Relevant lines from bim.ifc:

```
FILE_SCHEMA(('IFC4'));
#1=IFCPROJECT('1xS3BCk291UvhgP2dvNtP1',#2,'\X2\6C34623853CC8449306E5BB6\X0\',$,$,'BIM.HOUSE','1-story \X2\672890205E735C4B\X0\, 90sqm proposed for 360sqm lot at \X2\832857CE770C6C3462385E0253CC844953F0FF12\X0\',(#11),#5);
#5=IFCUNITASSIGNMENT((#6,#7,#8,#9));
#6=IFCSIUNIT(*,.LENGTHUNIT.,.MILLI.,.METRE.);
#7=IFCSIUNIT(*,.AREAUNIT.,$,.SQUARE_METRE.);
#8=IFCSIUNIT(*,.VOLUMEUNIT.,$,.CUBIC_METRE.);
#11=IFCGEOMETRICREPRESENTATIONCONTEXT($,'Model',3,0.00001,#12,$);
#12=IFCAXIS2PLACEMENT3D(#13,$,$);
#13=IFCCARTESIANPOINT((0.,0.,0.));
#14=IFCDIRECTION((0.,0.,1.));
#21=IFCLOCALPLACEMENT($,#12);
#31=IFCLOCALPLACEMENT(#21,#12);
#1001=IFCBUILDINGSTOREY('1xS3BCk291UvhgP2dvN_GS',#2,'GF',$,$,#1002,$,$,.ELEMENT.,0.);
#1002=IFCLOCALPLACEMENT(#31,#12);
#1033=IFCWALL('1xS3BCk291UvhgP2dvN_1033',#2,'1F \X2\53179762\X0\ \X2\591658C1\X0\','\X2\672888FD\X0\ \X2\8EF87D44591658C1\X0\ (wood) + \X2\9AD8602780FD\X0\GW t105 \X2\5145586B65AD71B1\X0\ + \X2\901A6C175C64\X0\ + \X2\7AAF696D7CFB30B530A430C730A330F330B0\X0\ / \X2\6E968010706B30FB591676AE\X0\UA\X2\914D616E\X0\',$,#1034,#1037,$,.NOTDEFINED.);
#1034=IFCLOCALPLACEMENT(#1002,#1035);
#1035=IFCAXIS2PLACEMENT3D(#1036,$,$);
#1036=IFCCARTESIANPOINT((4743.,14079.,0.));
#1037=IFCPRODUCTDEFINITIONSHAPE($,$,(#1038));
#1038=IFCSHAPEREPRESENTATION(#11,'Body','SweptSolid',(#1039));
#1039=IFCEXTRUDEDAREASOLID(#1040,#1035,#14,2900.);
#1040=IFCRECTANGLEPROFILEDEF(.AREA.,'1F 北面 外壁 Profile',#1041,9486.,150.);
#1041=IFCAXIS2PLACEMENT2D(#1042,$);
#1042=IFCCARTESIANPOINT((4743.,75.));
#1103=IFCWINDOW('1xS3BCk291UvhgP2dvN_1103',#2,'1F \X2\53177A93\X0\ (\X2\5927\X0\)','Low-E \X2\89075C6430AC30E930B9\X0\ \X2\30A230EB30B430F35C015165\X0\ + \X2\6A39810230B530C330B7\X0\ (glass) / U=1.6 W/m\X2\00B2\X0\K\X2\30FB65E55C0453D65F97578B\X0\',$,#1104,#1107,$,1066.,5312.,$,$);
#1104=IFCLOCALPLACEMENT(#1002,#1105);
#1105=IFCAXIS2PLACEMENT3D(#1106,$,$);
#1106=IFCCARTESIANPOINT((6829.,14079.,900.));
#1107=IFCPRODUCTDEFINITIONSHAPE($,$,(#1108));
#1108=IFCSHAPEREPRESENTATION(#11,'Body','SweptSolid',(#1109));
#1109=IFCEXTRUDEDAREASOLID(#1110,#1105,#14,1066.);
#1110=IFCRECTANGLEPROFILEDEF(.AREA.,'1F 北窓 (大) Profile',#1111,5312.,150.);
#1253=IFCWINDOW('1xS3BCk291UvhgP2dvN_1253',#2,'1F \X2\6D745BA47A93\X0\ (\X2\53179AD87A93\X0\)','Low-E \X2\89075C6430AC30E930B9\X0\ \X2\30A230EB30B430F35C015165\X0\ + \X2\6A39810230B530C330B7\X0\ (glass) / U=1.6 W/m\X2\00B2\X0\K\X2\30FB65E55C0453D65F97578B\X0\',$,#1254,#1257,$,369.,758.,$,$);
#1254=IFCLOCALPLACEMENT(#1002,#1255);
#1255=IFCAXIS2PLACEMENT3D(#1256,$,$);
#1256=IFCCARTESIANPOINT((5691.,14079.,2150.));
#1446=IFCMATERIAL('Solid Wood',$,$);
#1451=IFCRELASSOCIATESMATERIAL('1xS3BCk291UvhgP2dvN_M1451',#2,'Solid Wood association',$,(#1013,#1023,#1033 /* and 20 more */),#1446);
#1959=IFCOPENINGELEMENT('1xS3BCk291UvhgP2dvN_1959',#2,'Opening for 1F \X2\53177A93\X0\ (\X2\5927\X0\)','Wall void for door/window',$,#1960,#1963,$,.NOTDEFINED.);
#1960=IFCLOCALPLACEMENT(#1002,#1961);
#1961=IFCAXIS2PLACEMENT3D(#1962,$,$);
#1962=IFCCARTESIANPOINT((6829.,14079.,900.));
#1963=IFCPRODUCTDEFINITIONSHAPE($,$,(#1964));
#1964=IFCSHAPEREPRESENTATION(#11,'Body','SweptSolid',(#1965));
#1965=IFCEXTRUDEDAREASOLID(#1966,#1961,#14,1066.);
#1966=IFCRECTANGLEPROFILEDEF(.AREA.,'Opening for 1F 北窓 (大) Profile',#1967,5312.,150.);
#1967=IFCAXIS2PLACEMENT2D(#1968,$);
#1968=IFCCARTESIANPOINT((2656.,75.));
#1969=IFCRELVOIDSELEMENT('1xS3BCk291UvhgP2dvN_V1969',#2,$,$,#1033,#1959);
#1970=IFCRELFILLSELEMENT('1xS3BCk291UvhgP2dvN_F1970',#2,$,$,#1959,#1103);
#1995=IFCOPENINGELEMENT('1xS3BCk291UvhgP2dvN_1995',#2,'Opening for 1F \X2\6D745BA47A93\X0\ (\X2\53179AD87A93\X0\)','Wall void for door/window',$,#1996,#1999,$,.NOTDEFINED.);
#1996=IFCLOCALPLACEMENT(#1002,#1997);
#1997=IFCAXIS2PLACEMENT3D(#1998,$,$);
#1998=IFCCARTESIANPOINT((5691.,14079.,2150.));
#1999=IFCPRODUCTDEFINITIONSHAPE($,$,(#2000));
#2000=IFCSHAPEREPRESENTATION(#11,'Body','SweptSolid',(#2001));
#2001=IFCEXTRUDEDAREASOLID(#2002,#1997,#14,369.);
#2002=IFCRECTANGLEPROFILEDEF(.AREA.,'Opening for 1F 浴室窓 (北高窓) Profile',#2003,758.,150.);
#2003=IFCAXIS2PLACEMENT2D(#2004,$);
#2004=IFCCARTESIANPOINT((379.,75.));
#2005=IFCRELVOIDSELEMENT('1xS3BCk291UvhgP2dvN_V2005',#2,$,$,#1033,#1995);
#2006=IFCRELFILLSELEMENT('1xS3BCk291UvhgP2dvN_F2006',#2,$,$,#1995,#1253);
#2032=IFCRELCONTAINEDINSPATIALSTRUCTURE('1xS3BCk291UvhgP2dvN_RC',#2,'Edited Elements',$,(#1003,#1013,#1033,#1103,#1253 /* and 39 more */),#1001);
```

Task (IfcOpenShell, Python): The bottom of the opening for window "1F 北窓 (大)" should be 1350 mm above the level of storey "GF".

```python
import numpy as np
import ifcopenshell
import ifcopenshell.api.geometry
import ifcopenshell.geom
import ifcopenshell.util.element
import ifcopenshell.util.placement
import ifcopenshell.util.shape
import ifcopenshell.util.unit

model = ifcopenshell.open("bim.ifc")
unit_scale = ifcopenshell.util.unit.calculate_unit_scale(model)

window = model.by_id(1103)
opening = window.FillsVoids[0].RelatingOpeningElement
storey = ifcopenshell.util.element.get_container(window, ifc_class="IfcBuildingStorey")
level = ifcopenshell.util.placement.get_local_placement(storey.ObjectPlacement)[2, 3]

# The opening's origin need not be at the sill, so measure its lowest point.
shape = ifcopenshell.geom.create_shape(ifcopenshell.geom.settings(), opening)
bottom = ifcopenshell.util.shape.get_shape_bottom_elevation(shape, shape.geometry) / unit_scale
dz = level + 1.35 / unit_scale - bottom

shift = np.array([0.0, 0.0, dz])
# The window is not placed relative to its opening, so move both.
for product in (opening, window):
    matrix = ifcopenshell.util.placement.get_local_placement(product.ObjectPlacement)
    matrix[:3, 3] += shift
    ifcopenshell.api.geometry.edit_object_placement(model, product=product, matrix=matrix, is_si=False)

print(f"moved by {dz * unit_scale:+.3f} m")

model.write("bim_rev.ifc")
```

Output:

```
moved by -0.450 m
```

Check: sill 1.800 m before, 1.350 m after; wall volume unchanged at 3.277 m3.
